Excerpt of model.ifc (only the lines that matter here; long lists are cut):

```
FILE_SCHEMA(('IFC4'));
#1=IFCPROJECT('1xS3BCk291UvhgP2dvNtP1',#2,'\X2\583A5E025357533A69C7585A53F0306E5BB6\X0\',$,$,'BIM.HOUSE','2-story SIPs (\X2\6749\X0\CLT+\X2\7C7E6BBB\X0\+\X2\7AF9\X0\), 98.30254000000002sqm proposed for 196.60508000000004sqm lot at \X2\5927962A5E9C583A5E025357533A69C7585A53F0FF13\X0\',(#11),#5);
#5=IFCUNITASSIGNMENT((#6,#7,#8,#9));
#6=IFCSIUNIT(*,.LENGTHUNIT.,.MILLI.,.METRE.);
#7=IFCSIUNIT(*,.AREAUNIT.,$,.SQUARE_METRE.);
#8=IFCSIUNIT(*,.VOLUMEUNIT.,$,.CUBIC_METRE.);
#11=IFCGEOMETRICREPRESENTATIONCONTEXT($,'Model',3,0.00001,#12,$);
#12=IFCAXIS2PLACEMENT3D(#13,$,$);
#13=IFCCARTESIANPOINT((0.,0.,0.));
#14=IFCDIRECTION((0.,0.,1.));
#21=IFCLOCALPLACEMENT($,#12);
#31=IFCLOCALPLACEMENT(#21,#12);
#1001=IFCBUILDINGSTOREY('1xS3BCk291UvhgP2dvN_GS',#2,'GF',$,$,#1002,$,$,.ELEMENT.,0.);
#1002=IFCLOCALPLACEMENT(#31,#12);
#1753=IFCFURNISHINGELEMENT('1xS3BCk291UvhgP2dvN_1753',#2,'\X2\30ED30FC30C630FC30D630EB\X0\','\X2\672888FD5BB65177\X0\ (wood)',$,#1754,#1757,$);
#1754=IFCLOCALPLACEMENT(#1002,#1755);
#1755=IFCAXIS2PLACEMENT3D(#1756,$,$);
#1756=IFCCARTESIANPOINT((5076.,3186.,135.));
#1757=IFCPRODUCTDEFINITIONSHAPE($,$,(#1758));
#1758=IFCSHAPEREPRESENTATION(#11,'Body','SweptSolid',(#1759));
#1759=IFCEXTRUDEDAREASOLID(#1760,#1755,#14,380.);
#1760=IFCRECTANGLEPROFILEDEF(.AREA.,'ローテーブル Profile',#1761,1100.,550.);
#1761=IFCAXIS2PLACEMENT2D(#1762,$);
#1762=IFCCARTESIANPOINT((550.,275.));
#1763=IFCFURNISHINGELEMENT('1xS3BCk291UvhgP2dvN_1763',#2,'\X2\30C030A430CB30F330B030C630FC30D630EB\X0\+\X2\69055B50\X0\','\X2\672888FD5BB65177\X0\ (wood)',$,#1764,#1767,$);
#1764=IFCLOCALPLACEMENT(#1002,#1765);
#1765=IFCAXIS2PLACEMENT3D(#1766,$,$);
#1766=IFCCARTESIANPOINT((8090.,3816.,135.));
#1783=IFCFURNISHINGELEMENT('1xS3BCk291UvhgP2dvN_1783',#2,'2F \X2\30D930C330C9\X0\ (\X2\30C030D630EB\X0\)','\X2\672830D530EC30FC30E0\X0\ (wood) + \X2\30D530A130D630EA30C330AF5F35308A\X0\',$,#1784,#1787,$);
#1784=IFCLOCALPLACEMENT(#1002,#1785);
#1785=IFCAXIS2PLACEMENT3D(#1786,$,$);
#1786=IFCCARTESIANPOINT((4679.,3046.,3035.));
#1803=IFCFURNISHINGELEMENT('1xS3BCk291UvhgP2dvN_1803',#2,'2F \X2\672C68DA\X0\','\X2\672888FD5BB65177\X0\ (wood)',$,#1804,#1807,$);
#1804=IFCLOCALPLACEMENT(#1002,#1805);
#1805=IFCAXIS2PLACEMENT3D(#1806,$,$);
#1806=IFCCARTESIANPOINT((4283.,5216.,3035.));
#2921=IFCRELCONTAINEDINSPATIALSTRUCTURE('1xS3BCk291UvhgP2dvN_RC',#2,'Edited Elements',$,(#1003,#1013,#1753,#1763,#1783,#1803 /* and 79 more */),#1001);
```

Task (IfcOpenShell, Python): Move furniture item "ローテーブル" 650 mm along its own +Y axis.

```python
import ifcopenshell
import ifcopenshell.api.geometry
import ifcopenshell.util.placement
import ifcopenshell.util.unit

model = ifcopenshell.open("model.ifc")
unit_scale = ifcopenshell.util.unit.calculate_unit_scale(model)

item = model.by_guid("1xS3BCk291UvhgP2dvN_1753")
matrix = ifcopenshell.util.placement.get_local_placement(item.ObjectPlacement)
matrix[:3, 3] += matrix[:3, 1] * 0.65 / unit_scale
ifcopenshell.api.geometry.edit_object_placement(model, product=item, matrix=matrix, is_si=False)

print(ifcopenshell.util.placement.get_local_placement(item.ObjectPlacement).round(3) + 0.0)

model.write("model_updated.ifc")
```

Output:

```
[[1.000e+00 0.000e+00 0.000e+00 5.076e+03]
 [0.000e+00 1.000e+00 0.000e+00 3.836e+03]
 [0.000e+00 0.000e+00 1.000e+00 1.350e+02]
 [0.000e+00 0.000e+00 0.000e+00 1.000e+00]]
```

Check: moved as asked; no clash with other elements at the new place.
